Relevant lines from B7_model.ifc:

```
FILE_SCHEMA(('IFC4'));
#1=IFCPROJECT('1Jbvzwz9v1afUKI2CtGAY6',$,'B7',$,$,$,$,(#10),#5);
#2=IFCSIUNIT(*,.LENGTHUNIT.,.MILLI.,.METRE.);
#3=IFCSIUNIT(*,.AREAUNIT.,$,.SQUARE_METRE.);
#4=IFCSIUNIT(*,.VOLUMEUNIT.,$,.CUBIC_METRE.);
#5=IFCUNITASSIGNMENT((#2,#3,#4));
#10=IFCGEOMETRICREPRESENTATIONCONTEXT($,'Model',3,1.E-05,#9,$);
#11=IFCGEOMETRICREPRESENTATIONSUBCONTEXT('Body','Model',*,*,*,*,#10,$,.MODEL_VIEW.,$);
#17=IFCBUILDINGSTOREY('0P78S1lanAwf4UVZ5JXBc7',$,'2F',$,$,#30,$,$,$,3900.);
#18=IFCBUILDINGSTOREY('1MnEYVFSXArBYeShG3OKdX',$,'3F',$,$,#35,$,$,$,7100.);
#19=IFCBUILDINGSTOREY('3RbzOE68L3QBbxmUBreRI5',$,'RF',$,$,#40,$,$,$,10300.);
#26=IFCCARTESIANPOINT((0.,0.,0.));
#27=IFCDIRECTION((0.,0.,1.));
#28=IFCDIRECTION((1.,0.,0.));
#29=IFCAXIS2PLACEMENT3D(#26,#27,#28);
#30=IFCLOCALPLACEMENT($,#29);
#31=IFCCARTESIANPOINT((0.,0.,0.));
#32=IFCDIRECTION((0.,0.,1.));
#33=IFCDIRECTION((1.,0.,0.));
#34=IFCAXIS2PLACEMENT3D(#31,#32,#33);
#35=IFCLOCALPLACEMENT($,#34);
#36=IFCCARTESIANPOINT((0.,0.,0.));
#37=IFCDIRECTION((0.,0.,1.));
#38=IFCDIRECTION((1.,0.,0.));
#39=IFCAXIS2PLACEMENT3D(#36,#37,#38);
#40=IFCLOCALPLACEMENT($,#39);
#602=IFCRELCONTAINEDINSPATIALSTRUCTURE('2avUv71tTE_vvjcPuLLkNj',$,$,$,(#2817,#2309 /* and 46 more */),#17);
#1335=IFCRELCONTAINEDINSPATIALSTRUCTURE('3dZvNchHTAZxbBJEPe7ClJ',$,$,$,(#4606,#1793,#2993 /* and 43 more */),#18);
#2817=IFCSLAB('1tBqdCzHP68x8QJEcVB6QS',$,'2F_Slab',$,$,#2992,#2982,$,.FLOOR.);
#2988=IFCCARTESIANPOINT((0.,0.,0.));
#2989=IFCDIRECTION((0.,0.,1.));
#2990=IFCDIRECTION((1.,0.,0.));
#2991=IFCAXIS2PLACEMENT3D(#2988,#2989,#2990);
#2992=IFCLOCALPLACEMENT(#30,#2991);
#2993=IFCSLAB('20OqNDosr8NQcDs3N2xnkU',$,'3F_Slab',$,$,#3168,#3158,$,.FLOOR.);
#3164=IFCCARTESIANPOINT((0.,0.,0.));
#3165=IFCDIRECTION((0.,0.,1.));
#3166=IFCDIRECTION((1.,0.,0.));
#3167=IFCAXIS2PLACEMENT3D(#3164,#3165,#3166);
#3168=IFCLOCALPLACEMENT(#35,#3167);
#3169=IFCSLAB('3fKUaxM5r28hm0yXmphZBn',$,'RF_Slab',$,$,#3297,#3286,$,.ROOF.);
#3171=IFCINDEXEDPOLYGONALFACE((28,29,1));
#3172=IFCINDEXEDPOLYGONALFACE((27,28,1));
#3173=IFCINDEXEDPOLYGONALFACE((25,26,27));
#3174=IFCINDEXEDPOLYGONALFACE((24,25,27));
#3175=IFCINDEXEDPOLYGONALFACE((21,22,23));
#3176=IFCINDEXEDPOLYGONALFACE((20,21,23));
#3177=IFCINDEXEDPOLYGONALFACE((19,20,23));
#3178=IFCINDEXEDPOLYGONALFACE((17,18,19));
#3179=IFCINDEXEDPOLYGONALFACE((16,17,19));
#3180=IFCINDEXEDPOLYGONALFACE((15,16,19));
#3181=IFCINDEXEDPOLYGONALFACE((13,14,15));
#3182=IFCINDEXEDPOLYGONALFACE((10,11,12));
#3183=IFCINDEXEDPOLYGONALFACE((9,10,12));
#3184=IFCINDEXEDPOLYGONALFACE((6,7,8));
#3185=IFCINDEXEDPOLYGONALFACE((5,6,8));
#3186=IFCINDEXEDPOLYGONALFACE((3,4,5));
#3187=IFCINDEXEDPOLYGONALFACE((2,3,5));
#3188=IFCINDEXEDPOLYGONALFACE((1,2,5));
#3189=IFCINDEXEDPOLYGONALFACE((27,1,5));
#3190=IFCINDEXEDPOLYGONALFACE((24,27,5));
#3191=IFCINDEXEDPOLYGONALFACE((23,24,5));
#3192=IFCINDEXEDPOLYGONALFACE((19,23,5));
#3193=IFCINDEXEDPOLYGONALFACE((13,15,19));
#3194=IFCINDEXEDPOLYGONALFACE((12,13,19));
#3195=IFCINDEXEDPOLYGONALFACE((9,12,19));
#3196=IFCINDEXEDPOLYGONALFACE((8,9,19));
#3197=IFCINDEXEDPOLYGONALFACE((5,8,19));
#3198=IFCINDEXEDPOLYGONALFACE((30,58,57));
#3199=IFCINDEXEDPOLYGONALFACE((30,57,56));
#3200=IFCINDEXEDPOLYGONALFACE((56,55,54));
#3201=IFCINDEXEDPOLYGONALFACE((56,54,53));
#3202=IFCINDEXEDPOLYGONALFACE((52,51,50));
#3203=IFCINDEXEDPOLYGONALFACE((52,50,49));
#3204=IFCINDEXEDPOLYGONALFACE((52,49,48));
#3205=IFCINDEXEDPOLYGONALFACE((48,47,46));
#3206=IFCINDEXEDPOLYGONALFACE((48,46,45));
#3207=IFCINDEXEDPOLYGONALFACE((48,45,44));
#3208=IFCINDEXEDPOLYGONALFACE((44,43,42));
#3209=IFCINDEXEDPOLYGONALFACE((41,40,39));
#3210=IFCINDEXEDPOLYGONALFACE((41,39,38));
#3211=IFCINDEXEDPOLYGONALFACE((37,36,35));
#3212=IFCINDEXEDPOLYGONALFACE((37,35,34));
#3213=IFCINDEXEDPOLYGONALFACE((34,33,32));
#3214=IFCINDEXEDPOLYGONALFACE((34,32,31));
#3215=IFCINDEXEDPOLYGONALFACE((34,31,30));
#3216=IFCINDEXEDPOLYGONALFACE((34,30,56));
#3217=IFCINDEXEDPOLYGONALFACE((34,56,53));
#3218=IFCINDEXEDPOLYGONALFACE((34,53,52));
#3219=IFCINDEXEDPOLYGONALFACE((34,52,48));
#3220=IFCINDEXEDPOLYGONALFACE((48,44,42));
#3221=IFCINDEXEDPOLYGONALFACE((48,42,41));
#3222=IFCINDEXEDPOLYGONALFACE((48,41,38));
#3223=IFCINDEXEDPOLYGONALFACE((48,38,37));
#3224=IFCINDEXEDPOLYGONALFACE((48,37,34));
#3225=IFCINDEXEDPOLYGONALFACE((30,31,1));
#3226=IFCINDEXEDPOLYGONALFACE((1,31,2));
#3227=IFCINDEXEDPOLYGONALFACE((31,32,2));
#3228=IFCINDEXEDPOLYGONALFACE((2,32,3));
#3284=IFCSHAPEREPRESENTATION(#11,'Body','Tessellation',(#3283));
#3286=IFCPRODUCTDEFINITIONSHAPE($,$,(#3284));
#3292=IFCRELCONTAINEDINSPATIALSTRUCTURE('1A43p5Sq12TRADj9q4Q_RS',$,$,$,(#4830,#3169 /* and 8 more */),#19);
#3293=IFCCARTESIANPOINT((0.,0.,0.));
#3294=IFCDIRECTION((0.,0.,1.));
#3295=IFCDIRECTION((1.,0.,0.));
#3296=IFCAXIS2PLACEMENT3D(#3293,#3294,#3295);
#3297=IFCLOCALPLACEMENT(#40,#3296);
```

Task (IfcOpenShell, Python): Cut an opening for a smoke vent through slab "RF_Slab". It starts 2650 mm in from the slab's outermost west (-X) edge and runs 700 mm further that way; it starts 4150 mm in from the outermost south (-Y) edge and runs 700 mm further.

```python
import numpy as np
import ifcopenshell
import ifcopenshell.api.feature
import ifcopenshell.api.geometry
import ifcopenshell.api.root
import ifcopenshell.geom
import ifcopenshell.util.placement
import ifcopenshell.util.representation
import ifcopenshell.util.shape
import ifcopenshell.util.unit

model = ifcopenshell.open("B7_model.ifc")
unit_scale = ifcopenshell.util.unit.calculate_unit_scale(model)
settings = ifcopenshell.geom.settings()


def volume(element):
    """Net volume in cubic metres, openings subtracted."""
    shape = ifcopenshell.geom.create_shape(settings, element)
    return ifcopenshell.util.shape.get_volume(shape.geometry)


slab = model.by_guid("3fKUaxM5r28hm0yXmphZBn")
before = volume(slab)

# Extent in the slab's own axes, in metres. The edges named are its -X and -Y sides.
slab_shape = ifcopenshell.geom.create_shape(settings, slab)
vertices = ifcopenshell.util.shape.get_vertices(slab_shape.geometry)
x_min, y_min, bottom = vertices.min(axis=0)
top = vertices[:, 2].max()

opening = ifcopenshell.api.root.create_entity(model, ifc_class="IfcOpeningElement", name="Smoke vent opening", predefined_type="OPENING")
context = ifcopenshell.util.representation.get_context(model, "Model", "Body", "MODEL_VIEW")
width, depth = 0.7, 0.7
outline = [(0.0, 0.0), (width, 0.0), (width, depth), (0.0, depth), (0.0, 0.0)]
# Overshoot both faces by 50 mm so the cut is clean.
shape = ifcopenshell.api.geometry.add_slab_representation(
    model, context=context, depth=top - bottom + 0.1, polyline=outline
)
ifcopenshell.api.geometry.assign_representation(model, product=opening, representation=shape)

matrix = ifcopenshell.util.placement.get_local_placement(slab.ObjectPlacement)
matrix[:, 3] = matrix @ np.append(np.array([x_min + 2.65, y_min + 4.15, bottom - 0.05]) / unit_scale, 1.0)
ifcopenshell.api.geometry.edit_object_placement(model, product=opening, matrix=matrix, is_si=False)
ifcopenshell.api.feature.add_feature(model, feature=opening, element=slab)

after = volume(slab)

print(f"slab volume {before:.3f} -> {after:.3f} m3")

model.write("B7_model_v2.ifc")
```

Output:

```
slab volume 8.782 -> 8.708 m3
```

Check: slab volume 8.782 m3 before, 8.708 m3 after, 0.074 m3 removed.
